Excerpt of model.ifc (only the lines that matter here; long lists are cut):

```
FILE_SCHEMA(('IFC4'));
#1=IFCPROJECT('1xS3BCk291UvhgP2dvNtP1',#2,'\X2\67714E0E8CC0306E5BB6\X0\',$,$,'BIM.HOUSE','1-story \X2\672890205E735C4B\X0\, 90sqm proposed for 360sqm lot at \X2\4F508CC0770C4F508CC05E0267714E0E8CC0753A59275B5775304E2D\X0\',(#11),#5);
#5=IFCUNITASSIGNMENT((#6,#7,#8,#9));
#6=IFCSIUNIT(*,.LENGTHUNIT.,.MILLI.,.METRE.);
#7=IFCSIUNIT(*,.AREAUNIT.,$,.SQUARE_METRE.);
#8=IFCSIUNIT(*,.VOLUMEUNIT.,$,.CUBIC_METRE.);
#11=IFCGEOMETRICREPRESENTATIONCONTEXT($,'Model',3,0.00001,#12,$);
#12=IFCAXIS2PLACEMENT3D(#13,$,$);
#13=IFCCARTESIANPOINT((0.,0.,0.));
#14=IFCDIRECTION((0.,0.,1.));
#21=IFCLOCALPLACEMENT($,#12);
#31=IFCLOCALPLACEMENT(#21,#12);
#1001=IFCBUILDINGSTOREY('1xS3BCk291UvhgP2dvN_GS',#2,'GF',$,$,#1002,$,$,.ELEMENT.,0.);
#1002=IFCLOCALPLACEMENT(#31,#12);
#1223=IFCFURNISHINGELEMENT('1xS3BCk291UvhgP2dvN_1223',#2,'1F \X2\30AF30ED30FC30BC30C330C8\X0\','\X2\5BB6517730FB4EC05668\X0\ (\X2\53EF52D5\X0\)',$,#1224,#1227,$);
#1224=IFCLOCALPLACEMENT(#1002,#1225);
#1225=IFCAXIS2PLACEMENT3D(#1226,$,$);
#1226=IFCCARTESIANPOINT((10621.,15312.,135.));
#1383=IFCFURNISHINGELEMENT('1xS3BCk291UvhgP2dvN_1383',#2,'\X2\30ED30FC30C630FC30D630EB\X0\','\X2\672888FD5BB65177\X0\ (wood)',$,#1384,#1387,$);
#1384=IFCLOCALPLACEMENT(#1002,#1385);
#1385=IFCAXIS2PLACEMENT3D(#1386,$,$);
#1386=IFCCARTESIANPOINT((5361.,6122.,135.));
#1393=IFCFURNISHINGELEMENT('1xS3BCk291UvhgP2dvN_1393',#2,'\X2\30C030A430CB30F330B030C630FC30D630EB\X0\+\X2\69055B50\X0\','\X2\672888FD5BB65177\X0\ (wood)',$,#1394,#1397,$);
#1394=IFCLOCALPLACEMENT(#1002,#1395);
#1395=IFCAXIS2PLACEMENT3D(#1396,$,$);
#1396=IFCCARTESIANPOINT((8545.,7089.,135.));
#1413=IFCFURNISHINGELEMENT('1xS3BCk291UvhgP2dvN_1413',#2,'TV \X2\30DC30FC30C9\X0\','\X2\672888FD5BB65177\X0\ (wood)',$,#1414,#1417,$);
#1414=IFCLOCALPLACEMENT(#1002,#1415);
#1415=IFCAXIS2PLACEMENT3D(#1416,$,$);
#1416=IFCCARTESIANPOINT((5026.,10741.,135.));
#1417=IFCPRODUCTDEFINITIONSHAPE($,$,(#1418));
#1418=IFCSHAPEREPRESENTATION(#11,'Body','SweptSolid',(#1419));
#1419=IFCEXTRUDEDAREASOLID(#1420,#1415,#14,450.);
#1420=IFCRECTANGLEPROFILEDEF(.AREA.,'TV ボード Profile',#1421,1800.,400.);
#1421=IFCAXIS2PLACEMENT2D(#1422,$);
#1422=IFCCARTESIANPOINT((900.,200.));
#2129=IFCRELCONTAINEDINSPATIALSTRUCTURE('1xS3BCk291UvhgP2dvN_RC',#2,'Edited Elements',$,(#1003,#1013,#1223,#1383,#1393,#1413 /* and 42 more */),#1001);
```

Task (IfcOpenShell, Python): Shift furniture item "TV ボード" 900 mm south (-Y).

```python
import ifcopenshell
import ifcopenshell.api.geometry
import ifcopenshell.util.placement

model = ifcopenshell.open("model.ifc")

item = model.by_guid("1xS3BCk291UvhgP2dvN_1413")
matrix = ifcopenshell.util.placement.get_local_placement(item.ObjectPlacement)
matrix[1, 3] -= 900.0
ifcopenshell.api.geometry.edit_object_placement(model, product=item, matrix=matrix, is_si=False)

print(ifcopenshell.util.placement.get_local_placement(item.ObjectPlacement).round(3) + 0.0)

model.write("model_v2.ifc")
```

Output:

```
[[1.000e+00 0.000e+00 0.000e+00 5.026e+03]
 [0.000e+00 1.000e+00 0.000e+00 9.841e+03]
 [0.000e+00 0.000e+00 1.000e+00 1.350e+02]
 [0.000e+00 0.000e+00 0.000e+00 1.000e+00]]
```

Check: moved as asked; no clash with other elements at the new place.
